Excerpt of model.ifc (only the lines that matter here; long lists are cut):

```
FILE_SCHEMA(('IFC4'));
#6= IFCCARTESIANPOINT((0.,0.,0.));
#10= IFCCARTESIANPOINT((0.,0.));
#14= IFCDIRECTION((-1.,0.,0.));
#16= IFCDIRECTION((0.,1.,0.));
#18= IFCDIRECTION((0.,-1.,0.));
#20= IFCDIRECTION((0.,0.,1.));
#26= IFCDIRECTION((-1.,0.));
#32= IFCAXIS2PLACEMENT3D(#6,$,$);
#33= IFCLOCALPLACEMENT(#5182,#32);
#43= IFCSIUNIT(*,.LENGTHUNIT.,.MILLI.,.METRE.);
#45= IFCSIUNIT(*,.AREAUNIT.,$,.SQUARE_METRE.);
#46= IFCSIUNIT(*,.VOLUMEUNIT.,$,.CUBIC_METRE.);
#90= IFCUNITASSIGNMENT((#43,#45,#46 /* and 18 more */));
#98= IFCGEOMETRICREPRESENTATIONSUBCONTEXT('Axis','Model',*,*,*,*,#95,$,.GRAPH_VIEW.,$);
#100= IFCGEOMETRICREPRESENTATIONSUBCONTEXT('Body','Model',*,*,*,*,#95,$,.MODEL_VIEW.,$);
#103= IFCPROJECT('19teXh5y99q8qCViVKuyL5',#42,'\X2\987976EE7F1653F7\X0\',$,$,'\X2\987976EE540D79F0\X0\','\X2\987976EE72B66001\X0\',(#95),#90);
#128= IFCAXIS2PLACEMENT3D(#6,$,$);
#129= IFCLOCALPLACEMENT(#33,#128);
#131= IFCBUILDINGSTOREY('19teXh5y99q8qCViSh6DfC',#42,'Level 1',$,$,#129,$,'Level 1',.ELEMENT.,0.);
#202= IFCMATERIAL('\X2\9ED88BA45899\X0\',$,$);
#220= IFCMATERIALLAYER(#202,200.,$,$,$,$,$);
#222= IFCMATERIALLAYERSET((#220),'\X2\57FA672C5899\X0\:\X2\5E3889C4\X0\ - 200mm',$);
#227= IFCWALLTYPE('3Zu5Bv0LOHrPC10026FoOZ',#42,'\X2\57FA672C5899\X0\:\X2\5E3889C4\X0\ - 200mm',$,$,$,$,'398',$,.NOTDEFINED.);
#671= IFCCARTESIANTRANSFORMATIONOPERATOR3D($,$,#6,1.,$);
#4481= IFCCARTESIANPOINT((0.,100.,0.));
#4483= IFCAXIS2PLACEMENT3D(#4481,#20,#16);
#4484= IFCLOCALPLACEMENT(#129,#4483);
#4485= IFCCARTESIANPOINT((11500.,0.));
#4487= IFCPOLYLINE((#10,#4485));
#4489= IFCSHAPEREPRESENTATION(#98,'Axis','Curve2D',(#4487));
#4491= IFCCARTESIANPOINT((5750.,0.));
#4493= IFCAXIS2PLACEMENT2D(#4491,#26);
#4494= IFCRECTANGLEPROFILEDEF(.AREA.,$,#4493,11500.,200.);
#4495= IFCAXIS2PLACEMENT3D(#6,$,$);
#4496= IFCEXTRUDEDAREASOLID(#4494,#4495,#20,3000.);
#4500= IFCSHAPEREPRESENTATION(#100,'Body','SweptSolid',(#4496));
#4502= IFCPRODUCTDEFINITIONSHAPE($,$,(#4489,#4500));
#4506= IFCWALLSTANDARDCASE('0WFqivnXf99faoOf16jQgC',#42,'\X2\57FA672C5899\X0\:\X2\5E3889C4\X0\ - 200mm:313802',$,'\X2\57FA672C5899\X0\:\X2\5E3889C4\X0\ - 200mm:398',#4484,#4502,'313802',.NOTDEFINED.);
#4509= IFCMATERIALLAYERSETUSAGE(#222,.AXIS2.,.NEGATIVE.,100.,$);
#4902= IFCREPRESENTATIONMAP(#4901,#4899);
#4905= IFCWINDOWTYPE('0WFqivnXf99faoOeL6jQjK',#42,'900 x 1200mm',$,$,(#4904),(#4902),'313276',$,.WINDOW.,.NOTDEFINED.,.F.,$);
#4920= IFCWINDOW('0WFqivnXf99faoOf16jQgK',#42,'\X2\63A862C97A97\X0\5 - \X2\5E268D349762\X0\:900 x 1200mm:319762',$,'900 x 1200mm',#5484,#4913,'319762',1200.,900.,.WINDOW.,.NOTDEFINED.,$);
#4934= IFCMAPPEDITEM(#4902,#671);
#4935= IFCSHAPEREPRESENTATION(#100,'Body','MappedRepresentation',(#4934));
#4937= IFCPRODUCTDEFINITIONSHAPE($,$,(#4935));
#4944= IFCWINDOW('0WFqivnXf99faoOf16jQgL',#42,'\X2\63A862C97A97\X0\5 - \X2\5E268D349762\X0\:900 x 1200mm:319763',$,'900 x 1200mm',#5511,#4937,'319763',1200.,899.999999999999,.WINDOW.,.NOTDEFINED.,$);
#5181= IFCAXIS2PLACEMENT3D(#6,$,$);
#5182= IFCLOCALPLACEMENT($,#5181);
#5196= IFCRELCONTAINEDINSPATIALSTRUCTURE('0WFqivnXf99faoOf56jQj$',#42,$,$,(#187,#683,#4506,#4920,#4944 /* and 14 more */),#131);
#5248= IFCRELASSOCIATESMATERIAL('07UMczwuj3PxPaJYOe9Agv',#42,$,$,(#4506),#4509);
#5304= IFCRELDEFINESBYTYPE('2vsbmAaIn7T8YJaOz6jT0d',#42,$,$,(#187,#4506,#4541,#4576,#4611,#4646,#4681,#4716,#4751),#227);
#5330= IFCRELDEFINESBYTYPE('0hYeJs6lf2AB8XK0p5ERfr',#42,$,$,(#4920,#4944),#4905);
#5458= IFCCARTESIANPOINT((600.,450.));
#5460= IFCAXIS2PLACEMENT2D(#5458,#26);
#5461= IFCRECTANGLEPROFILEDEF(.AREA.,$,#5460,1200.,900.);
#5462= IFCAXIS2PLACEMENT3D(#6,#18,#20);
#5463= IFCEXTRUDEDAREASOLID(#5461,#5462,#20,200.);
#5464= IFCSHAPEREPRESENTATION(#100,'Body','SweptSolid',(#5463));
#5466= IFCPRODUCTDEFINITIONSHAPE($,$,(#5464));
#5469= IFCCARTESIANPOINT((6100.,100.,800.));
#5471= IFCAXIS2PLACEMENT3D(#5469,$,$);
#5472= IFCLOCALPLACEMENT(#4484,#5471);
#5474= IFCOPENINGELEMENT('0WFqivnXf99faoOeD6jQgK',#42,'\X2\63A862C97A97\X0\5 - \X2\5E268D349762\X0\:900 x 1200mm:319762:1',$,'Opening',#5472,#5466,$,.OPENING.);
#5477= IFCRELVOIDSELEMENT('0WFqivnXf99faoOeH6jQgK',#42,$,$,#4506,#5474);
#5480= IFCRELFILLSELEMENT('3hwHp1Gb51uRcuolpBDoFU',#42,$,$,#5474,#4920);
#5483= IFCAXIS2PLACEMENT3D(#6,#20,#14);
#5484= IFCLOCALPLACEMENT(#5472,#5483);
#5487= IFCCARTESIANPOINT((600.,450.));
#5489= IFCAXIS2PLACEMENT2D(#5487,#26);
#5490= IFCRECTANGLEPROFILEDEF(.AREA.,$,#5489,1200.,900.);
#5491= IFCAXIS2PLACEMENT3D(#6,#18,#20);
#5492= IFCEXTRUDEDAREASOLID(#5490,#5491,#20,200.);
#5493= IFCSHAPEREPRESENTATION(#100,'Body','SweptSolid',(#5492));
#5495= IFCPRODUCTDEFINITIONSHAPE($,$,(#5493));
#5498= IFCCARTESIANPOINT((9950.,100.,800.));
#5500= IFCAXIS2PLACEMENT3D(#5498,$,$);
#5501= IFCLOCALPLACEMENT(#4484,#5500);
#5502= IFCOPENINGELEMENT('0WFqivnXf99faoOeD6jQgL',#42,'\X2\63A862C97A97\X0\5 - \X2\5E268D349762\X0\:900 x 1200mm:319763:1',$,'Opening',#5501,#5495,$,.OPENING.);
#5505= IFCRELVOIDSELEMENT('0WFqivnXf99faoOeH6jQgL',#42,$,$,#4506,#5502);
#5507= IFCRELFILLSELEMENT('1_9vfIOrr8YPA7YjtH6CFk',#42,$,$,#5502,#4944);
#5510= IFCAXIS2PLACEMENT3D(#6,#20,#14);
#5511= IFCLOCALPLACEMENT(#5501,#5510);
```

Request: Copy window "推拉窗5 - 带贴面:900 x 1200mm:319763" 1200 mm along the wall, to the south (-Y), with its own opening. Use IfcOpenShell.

```python
import ifcopenshell
import ifcopenshell.api.feature
import ifcopenshell.api.geometry
import ifcopenshell.api.root
import ifcopenshell.geom
import ifcopenshell.util.element
import ifcopenshell.util.placement
import ifcopenshell.util.shape

model = ifcopenshell.open("model.ifc")
settings = ifcopenshell.geom.settings()


def volume(element):
    """Net volume in cubic metres, openings subtracted."""
    shape = ifcopenshell.geom.create_shape(settings, element)
    return ifcopenshell.util.shape.get_volume(shape.geometry)


def reuse_history(source, copy):
    """copy_class also copies each property set's owner history, people and application; keep the originals."""
    for rel in copy.IsDefinedBy:
        if rel.is_a("IfcRelDefinesByProperties") and (history := rel.RelatingPropertyDefinition.OwnerHistory):
            rel.RelatingPropertyDefinition.OwnerHistory = source.OwnerHistory
            ifcopenshell.util.element.remove_deep2(model, history)


window = model.by_guid("0WFqivnXf99faoOf16jQgL")
opening = window.FillsVoids[0].RelatingOpeningElement
wall = opening.VoidsElements[0].RelatingBuildingElement
before = volume(wall)
shift = ifcopenshell.util.placement.get_local_placement(wall.ObjectPlacement)[:3, 0] * -1200.0

# copy_class copies the void relationship, type, container and properties, but no geometry.
new_opening = ifcopenshell.api.root.copy_class(model, product=opening)
new_opening.Representation = ifcopenshell.util.element.copy_deep(
    model, opening.Representation, exclude=["IfcGeometricRepresentationContext", "IfcRepresentationMap"]
)
new_opening.Name = "推拉窗5 - 带贴面:900 x 1200mm"
new_window = ifcopenshell.api.root.copy_class(model, product=window)
new_window.Representation = ifcopenshell.util.element.copy_deep(
    model, window.Representation, exclude=["IfcGeometricRepresentationContext", "IfcRepresentationMap"]
)
new_window.Name = "推拉窗5 - 带贴面:900 x 1200mm"
new_window.Tag = None
reuse_history(window, new_window)
ifcopenshell.api.feature.add_filling(model, opening=new_opening, element=new_window)

for old, new in ((opening, new_opening), (window, new_window)):
    matrix = ifcopenshell.util.placement.get_local_placement(old.ObjectPlacement)
    matrix[:3, 3] += shift
    ifcopenshell.api.geometry.edit_object_placement(model, product=new, matrix=matrix, is_si=False)

after = volume(wall)

print(f"wall volume {before:.3f} -> {after:.3f} m3")

model.write("model_edited.ifc")
```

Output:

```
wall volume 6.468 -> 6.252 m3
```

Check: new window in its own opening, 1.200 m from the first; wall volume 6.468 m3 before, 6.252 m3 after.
